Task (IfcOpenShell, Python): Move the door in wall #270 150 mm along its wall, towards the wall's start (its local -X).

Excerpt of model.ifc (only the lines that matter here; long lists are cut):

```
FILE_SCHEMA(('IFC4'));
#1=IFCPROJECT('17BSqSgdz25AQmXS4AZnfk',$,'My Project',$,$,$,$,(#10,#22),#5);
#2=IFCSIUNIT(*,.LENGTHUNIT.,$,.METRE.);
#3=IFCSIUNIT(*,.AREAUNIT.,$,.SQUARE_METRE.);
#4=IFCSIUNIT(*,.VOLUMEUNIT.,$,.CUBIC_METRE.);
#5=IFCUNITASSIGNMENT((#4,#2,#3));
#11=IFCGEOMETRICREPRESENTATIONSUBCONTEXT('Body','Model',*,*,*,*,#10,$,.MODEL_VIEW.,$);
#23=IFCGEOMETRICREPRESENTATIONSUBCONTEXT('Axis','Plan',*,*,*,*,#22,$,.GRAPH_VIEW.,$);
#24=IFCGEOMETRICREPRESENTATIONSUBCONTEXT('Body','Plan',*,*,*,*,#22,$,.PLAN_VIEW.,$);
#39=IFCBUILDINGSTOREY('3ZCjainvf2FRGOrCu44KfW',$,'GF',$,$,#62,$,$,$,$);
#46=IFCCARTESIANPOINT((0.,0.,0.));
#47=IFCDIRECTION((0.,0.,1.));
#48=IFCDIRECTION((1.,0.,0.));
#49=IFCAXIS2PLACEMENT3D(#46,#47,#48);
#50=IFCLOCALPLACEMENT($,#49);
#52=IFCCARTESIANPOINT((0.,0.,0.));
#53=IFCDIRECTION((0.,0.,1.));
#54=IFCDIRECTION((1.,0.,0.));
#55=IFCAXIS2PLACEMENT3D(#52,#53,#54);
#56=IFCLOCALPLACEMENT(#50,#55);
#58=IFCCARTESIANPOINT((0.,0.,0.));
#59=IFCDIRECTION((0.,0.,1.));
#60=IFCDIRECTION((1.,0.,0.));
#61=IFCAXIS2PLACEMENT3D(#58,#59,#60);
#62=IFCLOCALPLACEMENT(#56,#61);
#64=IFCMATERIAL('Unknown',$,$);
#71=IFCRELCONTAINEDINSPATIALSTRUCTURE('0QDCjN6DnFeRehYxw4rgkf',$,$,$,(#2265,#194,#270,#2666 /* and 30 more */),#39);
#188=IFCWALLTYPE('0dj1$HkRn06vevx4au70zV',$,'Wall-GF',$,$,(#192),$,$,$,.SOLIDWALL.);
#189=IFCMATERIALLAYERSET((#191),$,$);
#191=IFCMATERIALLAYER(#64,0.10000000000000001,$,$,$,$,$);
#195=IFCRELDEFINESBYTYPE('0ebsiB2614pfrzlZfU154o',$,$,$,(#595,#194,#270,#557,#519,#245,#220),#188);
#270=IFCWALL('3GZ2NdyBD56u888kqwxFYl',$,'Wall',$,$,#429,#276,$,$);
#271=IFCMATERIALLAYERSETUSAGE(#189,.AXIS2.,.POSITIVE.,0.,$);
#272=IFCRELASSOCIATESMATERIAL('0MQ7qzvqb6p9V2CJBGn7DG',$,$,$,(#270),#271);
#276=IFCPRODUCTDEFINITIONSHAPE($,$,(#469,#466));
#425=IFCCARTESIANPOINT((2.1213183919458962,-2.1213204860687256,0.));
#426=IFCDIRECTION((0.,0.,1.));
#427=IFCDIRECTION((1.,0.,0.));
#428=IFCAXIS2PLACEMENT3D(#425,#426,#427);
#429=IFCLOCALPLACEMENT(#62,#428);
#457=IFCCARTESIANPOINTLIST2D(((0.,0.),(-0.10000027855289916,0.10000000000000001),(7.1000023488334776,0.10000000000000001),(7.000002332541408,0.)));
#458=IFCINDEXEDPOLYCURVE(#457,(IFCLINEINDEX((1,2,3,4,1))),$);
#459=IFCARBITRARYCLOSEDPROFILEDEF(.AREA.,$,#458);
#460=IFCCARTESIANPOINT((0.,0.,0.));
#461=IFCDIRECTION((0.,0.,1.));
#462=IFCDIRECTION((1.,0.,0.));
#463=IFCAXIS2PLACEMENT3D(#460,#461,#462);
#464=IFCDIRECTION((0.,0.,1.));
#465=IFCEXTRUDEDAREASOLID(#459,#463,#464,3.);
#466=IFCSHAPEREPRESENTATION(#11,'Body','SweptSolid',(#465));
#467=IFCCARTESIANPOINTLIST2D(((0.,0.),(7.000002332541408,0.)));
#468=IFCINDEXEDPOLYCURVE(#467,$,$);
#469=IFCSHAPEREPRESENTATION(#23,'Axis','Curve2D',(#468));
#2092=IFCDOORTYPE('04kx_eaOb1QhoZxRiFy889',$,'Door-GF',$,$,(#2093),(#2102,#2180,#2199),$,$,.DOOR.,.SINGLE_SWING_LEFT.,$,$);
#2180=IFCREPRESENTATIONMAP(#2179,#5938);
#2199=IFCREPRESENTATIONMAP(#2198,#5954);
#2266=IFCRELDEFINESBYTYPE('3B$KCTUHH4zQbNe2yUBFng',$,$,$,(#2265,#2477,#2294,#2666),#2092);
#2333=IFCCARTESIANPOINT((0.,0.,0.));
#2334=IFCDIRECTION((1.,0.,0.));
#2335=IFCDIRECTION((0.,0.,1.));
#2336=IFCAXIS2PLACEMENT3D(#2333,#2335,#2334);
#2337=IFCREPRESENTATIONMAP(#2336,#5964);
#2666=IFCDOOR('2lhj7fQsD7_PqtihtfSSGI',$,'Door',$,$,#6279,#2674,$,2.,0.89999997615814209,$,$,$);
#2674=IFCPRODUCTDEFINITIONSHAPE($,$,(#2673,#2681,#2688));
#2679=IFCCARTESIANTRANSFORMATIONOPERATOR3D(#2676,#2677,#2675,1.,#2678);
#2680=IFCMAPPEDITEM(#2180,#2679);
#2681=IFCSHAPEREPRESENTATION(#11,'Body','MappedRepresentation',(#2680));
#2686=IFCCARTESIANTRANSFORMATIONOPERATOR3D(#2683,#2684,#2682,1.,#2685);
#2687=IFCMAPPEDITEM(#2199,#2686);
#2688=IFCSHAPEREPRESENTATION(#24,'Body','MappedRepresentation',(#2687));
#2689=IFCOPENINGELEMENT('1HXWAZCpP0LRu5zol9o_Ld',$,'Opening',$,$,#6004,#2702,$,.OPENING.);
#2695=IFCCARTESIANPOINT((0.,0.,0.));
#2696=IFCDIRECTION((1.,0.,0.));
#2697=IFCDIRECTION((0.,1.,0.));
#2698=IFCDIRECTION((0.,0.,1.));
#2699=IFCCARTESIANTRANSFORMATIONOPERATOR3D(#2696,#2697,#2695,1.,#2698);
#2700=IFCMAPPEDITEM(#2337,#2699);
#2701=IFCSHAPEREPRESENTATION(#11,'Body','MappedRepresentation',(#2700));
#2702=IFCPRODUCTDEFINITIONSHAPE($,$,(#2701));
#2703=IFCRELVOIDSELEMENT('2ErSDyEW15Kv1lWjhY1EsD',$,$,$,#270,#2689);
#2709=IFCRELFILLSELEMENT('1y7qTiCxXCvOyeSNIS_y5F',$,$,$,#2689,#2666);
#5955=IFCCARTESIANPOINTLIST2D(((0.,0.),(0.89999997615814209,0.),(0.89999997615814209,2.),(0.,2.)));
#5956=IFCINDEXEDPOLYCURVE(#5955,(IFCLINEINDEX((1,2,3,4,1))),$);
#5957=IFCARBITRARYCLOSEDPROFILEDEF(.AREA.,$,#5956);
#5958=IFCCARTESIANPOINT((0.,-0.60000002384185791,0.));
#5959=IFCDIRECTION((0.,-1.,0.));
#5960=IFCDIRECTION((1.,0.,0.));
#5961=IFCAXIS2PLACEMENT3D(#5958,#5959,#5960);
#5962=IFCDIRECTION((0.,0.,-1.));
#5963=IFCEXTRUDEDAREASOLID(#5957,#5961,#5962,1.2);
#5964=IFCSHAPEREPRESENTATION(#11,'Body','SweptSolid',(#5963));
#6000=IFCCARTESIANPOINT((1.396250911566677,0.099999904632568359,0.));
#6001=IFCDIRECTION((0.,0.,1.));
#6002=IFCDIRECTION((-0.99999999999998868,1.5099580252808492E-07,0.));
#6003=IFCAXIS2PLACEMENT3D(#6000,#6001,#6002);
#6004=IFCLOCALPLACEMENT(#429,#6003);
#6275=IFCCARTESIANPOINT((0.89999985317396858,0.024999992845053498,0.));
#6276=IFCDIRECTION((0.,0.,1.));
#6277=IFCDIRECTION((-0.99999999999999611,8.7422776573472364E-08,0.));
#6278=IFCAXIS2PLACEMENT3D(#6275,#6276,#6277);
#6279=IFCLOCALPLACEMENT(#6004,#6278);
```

```python
import ifcopenshell
import ifcopenshell.api.geometry
import ifcopenshell.util.placement
import ifcopenshell.util.unit

model = ifcopenshell.open("model.ifc")
unit_scale = ifcopenshell.util.unit.calculate_unit_scale(model)

door = model.by_guid("2lhj7fQsD7_PqtihtfSSGI")
opening = door.FillsVoids[0].RelatingOpeningElement
wall = opening.VoidsElements[0].RelatingBuildingElement

wall_matrix = ifcopenshell.util.placement.get_local_placement(wall.ObjectPlacement)
shift = wall_matrix[:3, 0] * -0.15 / unit_scale
before = ifcopenshell.util.placement.get_local_placement(door.ObjectPlacement)[:3, 3].copy()

# The door is placed relative to its opening, so it follows when the opening moves.
matrix = ifcopenshell.util.placement.get_local_placement(opening.ObjectPlacement)
matrix[:3, 3] += shift
ifcopenshell.api.geometry.edit_object_placement(
    model, product=opening, matrix=matrix, is_si=False, should_transform_children=True
)

after = ifcopenshell.util.placement.get_local_placement(door.ObjectPlacement)[:3, 3]
print("door moved by", (after - before).round(3) + 0.0)

model.write("model_v2.ifc")
```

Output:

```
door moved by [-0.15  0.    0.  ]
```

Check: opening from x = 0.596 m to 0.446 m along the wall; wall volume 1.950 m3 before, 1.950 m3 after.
